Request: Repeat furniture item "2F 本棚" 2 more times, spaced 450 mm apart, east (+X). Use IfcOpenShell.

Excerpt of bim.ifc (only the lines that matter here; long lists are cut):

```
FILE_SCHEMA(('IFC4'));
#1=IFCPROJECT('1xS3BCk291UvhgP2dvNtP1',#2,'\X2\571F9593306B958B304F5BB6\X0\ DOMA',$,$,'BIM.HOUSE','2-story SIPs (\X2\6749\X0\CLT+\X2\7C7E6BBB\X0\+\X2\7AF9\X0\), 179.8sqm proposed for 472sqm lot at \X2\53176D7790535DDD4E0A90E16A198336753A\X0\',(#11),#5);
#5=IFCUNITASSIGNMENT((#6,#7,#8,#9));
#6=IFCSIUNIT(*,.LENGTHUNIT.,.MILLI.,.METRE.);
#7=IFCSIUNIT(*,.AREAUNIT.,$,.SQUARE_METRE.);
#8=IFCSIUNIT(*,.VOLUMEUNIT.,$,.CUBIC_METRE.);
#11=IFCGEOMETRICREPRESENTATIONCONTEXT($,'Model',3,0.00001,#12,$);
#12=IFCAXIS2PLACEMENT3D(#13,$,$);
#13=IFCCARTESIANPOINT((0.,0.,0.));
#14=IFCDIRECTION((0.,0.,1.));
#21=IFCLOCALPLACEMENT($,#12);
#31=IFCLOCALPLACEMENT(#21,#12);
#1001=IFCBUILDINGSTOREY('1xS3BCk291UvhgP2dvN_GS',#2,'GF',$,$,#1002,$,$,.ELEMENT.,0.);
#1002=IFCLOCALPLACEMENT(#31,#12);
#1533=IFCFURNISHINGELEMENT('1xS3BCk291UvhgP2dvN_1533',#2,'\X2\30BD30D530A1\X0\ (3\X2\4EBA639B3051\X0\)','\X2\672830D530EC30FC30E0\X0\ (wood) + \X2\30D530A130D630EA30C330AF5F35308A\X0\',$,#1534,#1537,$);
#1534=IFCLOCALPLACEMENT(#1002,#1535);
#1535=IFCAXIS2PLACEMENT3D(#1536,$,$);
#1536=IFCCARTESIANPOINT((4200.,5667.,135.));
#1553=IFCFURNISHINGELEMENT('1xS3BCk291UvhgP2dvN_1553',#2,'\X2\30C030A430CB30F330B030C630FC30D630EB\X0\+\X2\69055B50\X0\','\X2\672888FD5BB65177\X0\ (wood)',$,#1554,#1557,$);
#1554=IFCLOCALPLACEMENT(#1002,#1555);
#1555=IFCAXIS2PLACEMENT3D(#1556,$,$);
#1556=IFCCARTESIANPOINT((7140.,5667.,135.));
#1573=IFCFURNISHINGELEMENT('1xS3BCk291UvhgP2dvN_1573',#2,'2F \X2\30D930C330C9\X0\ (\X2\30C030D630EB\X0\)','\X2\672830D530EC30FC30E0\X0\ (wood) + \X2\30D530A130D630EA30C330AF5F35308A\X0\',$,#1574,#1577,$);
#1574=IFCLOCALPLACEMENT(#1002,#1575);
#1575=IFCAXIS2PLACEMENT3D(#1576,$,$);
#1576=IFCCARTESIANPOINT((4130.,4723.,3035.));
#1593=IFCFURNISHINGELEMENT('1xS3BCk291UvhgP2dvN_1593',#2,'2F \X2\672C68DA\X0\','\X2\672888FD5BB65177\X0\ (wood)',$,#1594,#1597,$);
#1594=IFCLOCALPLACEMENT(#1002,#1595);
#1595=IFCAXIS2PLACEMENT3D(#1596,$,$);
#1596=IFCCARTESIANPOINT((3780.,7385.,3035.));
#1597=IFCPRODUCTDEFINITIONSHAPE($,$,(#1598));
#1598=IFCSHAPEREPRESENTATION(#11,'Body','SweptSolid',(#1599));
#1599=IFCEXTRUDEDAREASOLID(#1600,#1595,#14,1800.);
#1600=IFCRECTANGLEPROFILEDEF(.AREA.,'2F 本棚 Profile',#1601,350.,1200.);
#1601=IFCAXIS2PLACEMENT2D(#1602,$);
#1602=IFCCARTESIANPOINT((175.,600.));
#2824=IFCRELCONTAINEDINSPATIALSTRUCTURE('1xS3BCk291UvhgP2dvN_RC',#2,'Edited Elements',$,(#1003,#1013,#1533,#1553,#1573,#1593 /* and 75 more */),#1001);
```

```python
import numpy as np
import ifcopenshell
import ifcopenshell.api.geometry
import ifcopenshell.api.root
import ifcopenshell.util.element
import ifcopenshell.util.placement

model = ifcopenshell.open("bim.ifc")


def reuse_history(source, copy):
    """copy_class also copies each property set's owner history, people and application; keep the originals."""
    for rel in copy.IsDefinedBy:
        if rel.is_a("IfcRelDefinesByProperties") and (history := rel.RelatingPropertyDefinition.OwnerHistory):
            rel.RelatingPropertyDefinition.OwnerHistory = source.OwnerHistory
            ifcopenshell.util.element.remove_deep2(model, history)


source = model.by_id(1593)
base = ifcopenshell.util.placement.get_local_placement(source.ObjectPlacement)
step = np.array([1.0, 0.0, 0.0]) * 450.0

for i in range(1, 3):
    copy = ifcopenshell.api.root.copy_class(model, product=source)
    copy.Representation = ifcopenshell.util.element.copy_deep(
        model, source.Representation, exclude=["IfcGeometricRepresentationContext", "IfcRepresentationMap"]
    )
    reuse_history(source, copy)
    matrix = base.copy()
    matrix[:3, 3] += i * step
    print("added at", matrix[:3, 3].round(3) + 0.0)
    ifcopenshell.api.geometry.edit_object_placement(model, product=copy, matrix=matrix, is_si=False)

model.write("bim_v2.ifc")
```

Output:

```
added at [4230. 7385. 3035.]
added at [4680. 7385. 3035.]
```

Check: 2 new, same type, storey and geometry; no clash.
